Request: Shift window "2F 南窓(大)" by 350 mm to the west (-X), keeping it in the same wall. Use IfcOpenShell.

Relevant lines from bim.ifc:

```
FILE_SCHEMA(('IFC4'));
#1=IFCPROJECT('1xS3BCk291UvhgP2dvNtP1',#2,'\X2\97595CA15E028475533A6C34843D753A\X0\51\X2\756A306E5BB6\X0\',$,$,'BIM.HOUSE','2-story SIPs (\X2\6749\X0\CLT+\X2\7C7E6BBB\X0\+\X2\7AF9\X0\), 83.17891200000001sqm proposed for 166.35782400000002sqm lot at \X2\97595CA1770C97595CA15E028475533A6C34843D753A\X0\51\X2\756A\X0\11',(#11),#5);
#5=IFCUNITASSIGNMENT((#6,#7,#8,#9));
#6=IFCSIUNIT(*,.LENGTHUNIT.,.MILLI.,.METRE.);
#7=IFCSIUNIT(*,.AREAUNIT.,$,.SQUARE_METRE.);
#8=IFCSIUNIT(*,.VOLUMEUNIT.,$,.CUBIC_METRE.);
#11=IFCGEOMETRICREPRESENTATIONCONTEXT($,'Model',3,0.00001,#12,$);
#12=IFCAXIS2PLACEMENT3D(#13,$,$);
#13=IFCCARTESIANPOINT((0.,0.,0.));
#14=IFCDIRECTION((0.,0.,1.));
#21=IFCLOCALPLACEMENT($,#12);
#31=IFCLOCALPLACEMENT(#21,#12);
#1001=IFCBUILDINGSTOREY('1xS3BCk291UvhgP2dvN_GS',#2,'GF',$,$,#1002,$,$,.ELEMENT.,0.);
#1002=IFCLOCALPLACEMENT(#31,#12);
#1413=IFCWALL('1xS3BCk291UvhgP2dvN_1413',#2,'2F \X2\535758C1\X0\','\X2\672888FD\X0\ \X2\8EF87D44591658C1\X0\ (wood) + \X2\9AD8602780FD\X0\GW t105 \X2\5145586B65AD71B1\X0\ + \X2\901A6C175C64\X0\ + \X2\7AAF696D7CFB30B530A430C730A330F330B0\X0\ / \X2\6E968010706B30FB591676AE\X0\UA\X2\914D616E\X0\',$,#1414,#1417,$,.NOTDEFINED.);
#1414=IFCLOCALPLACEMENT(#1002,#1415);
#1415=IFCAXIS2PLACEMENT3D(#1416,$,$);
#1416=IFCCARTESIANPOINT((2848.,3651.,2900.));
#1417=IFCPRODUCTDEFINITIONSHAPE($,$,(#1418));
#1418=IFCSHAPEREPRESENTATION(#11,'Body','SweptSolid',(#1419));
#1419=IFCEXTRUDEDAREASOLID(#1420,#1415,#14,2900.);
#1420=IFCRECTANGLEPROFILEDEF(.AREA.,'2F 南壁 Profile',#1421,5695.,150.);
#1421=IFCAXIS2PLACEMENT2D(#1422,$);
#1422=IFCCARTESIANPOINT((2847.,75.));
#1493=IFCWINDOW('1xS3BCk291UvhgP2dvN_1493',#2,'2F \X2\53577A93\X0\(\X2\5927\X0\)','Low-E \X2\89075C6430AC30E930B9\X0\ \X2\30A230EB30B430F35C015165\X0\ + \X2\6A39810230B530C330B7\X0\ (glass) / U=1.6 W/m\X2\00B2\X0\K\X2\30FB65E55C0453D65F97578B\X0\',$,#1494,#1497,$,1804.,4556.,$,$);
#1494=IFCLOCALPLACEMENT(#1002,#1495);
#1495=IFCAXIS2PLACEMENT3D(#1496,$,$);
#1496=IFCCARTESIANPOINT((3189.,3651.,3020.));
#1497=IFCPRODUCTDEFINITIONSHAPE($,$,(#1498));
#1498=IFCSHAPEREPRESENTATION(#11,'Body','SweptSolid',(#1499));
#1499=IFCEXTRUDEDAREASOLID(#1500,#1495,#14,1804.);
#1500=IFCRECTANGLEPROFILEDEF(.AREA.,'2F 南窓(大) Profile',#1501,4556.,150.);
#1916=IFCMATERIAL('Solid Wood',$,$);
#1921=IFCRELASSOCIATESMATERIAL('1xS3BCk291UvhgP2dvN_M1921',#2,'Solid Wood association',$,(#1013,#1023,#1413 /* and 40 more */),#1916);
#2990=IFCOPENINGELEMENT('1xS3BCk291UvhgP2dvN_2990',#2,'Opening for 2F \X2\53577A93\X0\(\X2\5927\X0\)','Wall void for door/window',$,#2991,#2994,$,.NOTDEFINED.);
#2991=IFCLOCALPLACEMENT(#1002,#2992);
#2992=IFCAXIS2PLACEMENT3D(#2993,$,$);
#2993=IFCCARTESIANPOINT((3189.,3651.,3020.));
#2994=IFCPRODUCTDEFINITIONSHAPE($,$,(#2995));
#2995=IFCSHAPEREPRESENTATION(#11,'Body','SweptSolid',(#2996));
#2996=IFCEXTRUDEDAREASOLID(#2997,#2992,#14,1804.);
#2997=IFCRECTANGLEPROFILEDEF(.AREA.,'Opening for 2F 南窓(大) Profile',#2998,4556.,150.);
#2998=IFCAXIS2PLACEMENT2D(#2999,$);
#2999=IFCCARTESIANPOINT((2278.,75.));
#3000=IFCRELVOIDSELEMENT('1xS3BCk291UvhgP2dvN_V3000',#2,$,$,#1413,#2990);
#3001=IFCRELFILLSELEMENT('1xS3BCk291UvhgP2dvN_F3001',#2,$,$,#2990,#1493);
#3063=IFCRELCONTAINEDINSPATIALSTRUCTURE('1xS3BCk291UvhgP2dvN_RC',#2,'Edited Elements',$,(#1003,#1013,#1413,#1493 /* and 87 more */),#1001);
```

```python
import ifcopenshell
import ifcopenshell.api.geometry
import ifcopenshell.util.placement

model = ifcopenshell.open("bim.ifc")

window = model.by_guid("1xS3BCk291UvhgP2dvN_1493")
opening = window.FillsVoids[0].RelatingOpeningElement
wall = opening.VoidsElements[0].RelatingBuildingElement

wall_matrix = ifcopenshell.util.placement.get_local_placement(wall.ObjectPlacement)
shift = wall_matrix[:3, 0] * -350.0
before = ifcopenshell.util.placement.get_local_placement(window.ObjectPlacement)[:3, 3].copy()

# The window is not placed relative to its opening, so move both.
for product in (opening, window):
    matrix = ifcopenshell.util.placement.get_local_placement(product.ObjectPlacement)
    matrix[:3, 3] += shift
    ifcopenshell.api.geometry.edit_object_placement(model, product=product, matrix=matrix, is_si=False)

after = ifcopenshell.util.placement.get_local_placement(window.ObjectPlacement)[:3, 3]
print("window moved by", (after - before).round(3) + 0.0)

model.write("bim_v2.ifc")
```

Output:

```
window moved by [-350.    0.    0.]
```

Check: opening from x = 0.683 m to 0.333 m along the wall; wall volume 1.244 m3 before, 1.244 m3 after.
